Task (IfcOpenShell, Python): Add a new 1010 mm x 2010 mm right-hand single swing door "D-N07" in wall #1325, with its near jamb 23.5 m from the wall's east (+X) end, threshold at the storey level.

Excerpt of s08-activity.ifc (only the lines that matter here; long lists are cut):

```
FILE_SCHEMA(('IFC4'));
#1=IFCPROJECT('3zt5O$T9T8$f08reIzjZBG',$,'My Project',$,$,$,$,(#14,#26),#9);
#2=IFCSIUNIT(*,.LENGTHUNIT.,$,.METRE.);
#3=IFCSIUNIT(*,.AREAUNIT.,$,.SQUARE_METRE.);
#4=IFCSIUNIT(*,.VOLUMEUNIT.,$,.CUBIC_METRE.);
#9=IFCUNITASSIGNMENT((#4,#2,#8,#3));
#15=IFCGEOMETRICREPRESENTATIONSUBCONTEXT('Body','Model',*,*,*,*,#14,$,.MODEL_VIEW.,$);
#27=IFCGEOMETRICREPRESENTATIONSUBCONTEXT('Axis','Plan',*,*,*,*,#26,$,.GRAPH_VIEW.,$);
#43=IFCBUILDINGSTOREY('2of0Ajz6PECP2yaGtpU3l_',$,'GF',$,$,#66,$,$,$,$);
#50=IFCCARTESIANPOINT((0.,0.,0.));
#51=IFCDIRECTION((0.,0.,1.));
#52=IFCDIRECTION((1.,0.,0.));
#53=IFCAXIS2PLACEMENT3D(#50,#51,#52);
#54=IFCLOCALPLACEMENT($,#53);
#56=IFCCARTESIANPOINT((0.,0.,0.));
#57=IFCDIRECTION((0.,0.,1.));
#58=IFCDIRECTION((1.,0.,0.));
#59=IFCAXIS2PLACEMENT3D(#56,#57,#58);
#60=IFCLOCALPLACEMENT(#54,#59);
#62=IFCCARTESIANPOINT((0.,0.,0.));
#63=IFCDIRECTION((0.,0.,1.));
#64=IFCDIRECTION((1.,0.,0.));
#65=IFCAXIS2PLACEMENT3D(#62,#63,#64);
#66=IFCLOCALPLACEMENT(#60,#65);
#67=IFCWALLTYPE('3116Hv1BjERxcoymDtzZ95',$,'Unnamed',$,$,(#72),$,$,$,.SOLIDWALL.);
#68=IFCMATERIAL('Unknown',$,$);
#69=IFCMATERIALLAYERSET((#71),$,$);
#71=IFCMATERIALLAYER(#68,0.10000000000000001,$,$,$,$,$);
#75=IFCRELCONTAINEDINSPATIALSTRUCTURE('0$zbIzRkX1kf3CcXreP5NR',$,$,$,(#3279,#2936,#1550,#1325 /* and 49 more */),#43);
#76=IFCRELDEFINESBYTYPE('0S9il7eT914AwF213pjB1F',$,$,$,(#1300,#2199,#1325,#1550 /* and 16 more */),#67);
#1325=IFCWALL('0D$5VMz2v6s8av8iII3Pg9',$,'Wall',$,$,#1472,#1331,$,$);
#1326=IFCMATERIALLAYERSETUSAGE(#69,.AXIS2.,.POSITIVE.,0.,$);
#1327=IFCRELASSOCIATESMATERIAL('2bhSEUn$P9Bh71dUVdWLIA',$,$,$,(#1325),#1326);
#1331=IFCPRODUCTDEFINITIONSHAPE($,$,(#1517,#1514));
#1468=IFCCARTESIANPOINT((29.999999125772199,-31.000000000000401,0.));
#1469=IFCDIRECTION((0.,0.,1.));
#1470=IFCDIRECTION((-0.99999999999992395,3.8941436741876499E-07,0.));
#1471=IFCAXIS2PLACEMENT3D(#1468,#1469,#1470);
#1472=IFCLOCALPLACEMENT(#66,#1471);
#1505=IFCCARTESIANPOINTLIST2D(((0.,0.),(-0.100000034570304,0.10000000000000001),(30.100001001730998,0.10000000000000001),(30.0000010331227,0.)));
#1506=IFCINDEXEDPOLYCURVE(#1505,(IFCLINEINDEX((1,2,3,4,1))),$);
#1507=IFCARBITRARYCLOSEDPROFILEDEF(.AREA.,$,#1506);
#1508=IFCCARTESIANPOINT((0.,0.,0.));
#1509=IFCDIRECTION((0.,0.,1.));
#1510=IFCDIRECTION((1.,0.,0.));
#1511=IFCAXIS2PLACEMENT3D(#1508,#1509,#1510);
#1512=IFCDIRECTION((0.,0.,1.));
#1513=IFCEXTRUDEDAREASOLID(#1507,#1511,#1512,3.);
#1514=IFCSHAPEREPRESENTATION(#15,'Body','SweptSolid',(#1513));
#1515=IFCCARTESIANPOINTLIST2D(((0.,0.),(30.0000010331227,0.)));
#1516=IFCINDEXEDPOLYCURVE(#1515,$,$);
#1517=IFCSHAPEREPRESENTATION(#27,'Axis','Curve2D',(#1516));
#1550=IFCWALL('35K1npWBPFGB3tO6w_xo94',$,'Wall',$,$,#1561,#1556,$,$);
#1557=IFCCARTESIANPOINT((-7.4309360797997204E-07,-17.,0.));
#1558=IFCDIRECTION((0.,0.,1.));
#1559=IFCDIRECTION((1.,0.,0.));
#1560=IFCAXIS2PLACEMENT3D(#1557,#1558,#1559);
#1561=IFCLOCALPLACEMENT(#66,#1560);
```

```python
import numpy as np
import ifcopenshell
import ifcopenshell.api.feature
import ifcopenshell.api.geometry
import ifcopenshell.api.root
import ifcopenshell.api.spatial
import ifcopenshell.geom
import ifcopenshell.util.element
import ifcopenshell.util.placement
import ifcopenshell.util.representation
import ifcopenshell.util.shape
import ifcopenshell.util.unit

model = ifcopenshell.open("s08-activity.ifc")
unit_scale = ifcopenshell.util.unit.calculate_unit_scale(model)
settings = ifcopenshell.geom.settings()


def volume(element):
    """Net volume in cubic metres, openings subtracted."""
    shape = ifcopenshell.geom.create_shape(settings, element)
    return ifcopenshell.util.shape.get_volume(shape.geometry)


wall = model.by_guid("0D$5VMz2v6s8av8iII3Pg9")
storey = ifcopenshell.util.element.get_container(wall, ifc_class="IfcBuildingStorey")
context = ifcopenshell.util.representation.get_context(model, "Model", "Body", "MODEL_VIEW")
before = volume(wall)

width, height, from_end, sill = 1.01, 2.01, 23.5, 0.0  # metres

# The wall runs along its own X axis, and the end named is its -X end.
wall_shape = ifcopenshell.geom.create_shape(settings, wall)
x, y, z = ifcopenshell.util.shape.get_vertices(wall_shape.geometry).T
start = x.min() + from_end
face, thickness = float(y.min()), float(y.max() - y.min())
wall_matrix = ifcopenshell.util.placement.get_local_placement(wall.ObjectPlacement)
level = ifcopenshell.util.placement.get_local_placement(storey.ObjectPlacement)[2, 3]


def in_wall(x, y):
    """Placement at x, y metres in the wall's axes, at sill height."""
    matrix = wall_matrix.copy()
    matrix[:, 3] = wall_matrix @ np.array([x / unit_scale, y / unit_scale, 0.0, 1.0])
    matrix[2, 3] = level + sill / unit_scale
    return matrix


# Opening: a box that overshoots both wall faces by 50 mm.
opening = ifcopenshell.api.root.create_entity(model, ifc_class="IfcOpeningElement", predefined_type="OPENING")
box = ifcopenshell.api.geometry.add_wall_representation(
    model, context=context, length=width, height=height, thickness=thickness + 0.1
)
ifcopenshell.api.geometry.assign_representation(model, product=opening, representation=box)
ifcopenshell.api.geometry.edit_object_placement(model, product=opening, matrix=in_wall(start, face - 0.05), is_si=False)
ifcopenshell.api.feature.add_feature(model, feature=opening, element=wall)

door = ifcopenshell.api.root.create_entity(model, ifc_class="IfcDoor", name="D-N07", predefined_type="DOOR")
door.OverallWidth, door.OverallHeight = width / unit_scale, height / unit_scale
door.OperationType = "SINGLE_SWING_RIGHT"
body = ifcopenshell.api.geometry.add_door_representation(
    model,
    context=context,
    overall_width=door.OverallWidth,
    overall_height=door.OverallHeight,
    operation_type="SINGLE_SWING_RIGHT",
    lining_properties={"LiningDepth": thickness / unit_scale, "ThresholdDepth": thickness / unit_scale},
)
ifcopenshell.api.geometry.assign_representation(model, product=door, representation=body)
ifcopenshell.api.spatial.assign_container(model, products=[door], relating_structure=storey)
ifcopenshell.api.feature.add_filling(model, opening=opening, element=door)

# The lining spans the wall, so the door starts at the wall face.
ifcopenshell.api.geometry.edit_object_placement(model, product=door, matrix=in_wall(start, face), is_si=False)

after = volume(wall)

print(f"wall volume {before:.3f} -> {after:.3f} m3")

model.write("s08-activity_updated.ifc")
```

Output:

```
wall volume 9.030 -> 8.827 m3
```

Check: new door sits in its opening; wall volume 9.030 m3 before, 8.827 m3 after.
